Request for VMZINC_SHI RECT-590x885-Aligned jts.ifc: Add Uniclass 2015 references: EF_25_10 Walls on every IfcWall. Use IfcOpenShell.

First a look at what the model holds.

```python
import ifcopenshell

model = ifcopenshell.open("VMZINC_SHI RECT-590x885-Aligned jts.ifc")
print(model.schema)
print("classifications:", [c.Name for c in model.by_type("IfcClassification")])
for ifc_class in ("IfcDoor", "IfcRoof", "IfcStair", "IfcWall", "IfcWindow"):
    print(ifc_class, len(model.by_type(ifc_class)))
```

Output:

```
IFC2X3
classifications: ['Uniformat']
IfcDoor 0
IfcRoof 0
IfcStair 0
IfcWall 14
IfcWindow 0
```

```python
import ifcopenshell
import ifcopenshell.api.classification

model = ifcopenshell.open("VMZINC_SHI RECT-590x885-Aligned jts.ifc")

# IFC2X3 requires Source and Edition and has no link from the project to the system.
system = model.create_entity("IfcClassification", Source="NBS", Edition="2015", Name="Uniclass 2015")

codes = {
    "IfcWall": ("EF_25_10", "Walls"),
}
for ifc_class, (code, name) in codes.items():
    products = model.by_type(ifc_class)
    ifcopenshell.api.classification.add_reference(
        model, products=products, classification=system, identification=code, name=name
    )
    print(code, len(products))

model.write("VMZINC_SHI RECT-590x885-Aligned jts_updated.ifc")
```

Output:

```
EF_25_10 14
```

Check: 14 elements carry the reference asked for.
